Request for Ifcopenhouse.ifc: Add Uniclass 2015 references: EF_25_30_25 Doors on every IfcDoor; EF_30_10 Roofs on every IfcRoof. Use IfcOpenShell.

First a look at what the model holds.

```python
import ifcopenshell

model = ifcopenshell.open("Ifcopenhouse.ifc")
print(model.schema)
print("classifications:", [c.Name for c in model.by_type("IfcClassification")])
for ifc_class in ("IfcDoor", "IfcRoof", "IfcStair", "IfcWall", "IfcWindow"):
    print(ifc_class, len(model.by_type(ifc_class)))
```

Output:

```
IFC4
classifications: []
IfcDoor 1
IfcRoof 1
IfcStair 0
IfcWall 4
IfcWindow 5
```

```python
import ifcopenshell
import ifcopenshell.api.classification

model = ifcopenshell.open("Ifcopenhouse.ifc")

system = ifcopenshell.api.classification.add_classification(model, classification="Uniclass 2015")

codes = {
    "IfcDoor": ("EF_25_30_25", "Doors"),
    "IfcRoof": ("EF_30_10", "Roofs"),
}
for ifc_class, (code, name) in codes.items():
    products = model.by_type(ifc_class)
    ifcopenshell.api.classification.add_reference(
        model, products=products, classification=system, identification=code, name=name
    )
    print(code, len(products))

model.write("Ifcopenhouse_updated.ifc")
```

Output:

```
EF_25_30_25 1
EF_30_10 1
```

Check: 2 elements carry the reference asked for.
